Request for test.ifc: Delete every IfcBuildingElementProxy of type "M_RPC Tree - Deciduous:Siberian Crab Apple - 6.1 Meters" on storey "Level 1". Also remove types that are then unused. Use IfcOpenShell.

First a look at what the model holds.

```python
import ifcopenshell
import ifcopenshell.util.element

model = ifcopenshell.open("test.ifc")
print(model.schema)
storey = next(s for s in model.by_type("IfcBuildingStorey") if s.Name == "Level 1")
proxies = [e for e in ifcopenshell.util.element.get_decomposition(storey) if e.is_a("IfcBuildingElementProxy")]
seen = {}
for e in proxies:
    element_type = ifcopenshell.util.element.get_type(e)
    name = element_type.Name if element_type not in (None, e) else None
    seen[name] = seen.get(name, 0) + 1
for name, count in sorted(seen.items(), key=str):
    print(count, "x", name)
```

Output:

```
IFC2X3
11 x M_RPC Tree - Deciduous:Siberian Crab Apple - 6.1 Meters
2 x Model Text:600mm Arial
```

```python
import ifcopenshell
import ifcopenshell.api.root
import ifcopenshell.util.element

model = ifcopenshell.open("test.ifc")

storey = next(s for s in model.by_type("IfcBuildingStorey") if s.Name == "Level 1")
proxies = [e for e in ifcopenshell.util.element.get_decomposition(storey) if e.is_a("IfcBuildingElementProxy")]
targets = [e for e in proxies if (t := ifcopenshell.util.element.get_type(e)) not in (None, e) and t.Name == "M_RPC Tree - Deciduous:Siberian Crab Apple - 6.1 Meters"]
types = {ifcopenshell.util.element.get_type(e) for e in targets} - {None, *targets}

for e in targets:
    ifcopenshell.api.root.remove_product(model, product=e)
print(len(targets), "removed")

unused = [t for t in types if not ifcopenshell.util.element.get_types(t)]
for t in unused:
    ifcopenshell.api.root.remove_product(model, product=t)
print(len(unused), "unused types removed")

model.write("test_edited.ifc")
```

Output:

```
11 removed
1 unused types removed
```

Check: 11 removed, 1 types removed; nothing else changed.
